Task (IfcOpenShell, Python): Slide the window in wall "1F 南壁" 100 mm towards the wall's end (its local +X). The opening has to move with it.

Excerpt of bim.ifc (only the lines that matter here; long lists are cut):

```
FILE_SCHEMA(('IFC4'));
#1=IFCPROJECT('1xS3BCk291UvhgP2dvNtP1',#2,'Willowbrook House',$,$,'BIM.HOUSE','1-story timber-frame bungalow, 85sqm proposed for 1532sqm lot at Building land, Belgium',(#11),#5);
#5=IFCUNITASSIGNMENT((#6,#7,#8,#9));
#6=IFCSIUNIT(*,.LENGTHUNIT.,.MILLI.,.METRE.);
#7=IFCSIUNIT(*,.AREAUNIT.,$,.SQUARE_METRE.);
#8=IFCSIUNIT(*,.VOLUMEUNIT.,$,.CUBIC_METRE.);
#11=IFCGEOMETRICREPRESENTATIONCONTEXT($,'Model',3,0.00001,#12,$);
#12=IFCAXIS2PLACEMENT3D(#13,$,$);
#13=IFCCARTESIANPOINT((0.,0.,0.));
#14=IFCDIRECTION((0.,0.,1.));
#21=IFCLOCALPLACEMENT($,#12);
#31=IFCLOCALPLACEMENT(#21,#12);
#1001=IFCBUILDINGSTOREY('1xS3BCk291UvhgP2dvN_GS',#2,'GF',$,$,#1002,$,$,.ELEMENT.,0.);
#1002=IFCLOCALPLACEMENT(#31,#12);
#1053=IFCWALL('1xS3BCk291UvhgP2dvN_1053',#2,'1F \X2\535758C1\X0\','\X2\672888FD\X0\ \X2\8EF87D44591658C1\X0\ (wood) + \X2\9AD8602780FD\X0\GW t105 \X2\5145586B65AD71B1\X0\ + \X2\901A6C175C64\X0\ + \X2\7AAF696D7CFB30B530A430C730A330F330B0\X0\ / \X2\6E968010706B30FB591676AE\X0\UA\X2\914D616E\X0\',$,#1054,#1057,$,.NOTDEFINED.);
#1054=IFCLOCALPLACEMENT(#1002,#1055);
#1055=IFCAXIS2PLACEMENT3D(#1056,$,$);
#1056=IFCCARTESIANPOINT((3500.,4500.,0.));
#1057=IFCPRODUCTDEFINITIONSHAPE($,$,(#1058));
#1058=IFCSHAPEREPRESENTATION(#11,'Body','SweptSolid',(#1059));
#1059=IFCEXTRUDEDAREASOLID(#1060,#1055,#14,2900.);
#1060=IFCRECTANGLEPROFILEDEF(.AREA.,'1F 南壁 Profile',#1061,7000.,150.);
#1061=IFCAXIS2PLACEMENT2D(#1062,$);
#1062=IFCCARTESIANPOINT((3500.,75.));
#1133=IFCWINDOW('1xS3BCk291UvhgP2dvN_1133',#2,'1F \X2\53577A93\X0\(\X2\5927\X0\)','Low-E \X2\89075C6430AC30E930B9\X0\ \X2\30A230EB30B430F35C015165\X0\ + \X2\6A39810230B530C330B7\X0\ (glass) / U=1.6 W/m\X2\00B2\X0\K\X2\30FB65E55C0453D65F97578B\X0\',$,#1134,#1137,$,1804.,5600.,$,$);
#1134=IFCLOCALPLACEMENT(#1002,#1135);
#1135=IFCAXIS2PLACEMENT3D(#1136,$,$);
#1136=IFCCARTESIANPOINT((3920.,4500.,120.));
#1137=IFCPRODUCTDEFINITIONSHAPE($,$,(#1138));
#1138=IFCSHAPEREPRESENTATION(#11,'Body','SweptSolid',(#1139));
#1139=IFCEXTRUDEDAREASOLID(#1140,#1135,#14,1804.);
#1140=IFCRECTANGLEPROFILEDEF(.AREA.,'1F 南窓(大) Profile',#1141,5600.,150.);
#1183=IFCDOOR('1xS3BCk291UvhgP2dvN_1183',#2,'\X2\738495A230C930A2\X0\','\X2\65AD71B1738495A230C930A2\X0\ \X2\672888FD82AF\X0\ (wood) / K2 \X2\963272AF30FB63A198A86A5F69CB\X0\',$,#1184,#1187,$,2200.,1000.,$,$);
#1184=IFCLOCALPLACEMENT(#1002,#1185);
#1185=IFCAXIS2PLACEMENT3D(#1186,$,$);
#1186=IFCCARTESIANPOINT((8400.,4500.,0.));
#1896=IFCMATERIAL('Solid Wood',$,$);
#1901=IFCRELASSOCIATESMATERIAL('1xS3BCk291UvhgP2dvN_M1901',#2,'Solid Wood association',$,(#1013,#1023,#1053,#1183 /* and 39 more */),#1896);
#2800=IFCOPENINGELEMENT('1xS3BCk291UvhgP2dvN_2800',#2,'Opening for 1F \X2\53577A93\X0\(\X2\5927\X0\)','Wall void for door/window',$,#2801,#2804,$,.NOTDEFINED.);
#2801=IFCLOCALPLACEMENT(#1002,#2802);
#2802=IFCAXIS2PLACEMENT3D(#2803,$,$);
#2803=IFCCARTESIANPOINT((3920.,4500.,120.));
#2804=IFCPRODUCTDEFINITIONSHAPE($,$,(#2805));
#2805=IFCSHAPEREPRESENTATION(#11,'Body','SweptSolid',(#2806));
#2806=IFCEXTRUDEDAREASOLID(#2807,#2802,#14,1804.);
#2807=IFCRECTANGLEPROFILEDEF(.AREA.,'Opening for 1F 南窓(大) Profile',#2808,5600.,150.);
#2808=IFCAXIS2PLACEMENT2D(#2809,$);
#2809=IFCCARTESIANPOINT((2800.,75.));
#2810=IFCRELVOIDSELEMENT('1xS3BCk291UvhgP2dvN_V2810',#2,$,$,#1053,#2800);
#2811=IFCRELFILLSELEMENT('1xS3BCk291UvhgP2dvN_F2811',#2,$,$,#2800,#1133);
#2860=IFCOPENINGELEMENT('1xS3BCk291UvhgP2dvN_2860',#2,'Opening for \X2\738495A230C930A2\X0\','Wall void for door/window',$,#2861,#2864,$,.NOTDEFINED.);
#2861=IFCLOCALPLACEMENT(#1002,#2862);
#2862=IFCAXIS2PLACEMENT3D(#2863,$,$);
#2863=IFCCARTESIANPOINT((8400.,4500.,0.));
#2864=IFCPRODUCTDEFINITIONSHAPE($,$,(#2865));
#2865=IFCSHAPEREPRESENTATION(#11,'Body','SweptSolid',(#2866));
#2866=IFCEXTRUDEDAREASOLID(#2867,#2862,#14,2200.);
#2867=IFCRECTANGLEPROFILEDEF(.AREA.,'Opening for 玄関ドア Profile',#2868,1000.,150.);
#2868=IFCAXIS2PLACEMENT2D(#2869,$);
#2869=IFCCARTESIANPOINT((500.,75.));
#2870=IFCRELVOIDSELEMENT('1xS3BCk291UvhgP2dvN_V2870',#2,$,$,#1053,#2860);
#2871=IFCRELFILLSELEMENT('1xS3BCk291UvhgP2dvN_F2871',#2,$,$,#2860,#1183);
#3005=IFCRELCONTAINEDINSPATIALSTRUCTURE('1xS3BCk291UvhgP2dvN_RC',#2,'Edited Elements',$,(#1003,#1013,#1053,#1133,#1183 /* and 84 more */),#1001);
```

```python
import ifcopenshell
import ifcopenshell.api.geometry
import ifcopenshell.util.placement
import ifcopenshell.util.unit

model = ifcopenshell.open("bim.ifc")
unit_scale = ifcopenshell.util.unit.calculate_unit_scale(model)

window = model.by_id(1133)
opening = window.FillsVoids[0].RelatingOpeningElement
wall = opening.VoidsElements[0].RelatingBuildingElement

wall_matrix = ifcopenshell.util.placement.get_local_placement(wall.ObjectPlacement)
shift = wall_matrix[:3, 0] * 0.1 / unit_scale
before = ifcopenshell.util.placement.get_local_placement(window.ObjectPlacement)[:3, 3].copy()

# The window is not placed relative to its opening, so move both.
for product in (opening, window):
    matrix = ifcopenshell.util.placement.get_local_placement(product.ObjectPlacement)
    matrix[:3, 3] += shift
    ifcopenshell.api.geometry.edit_object_placement(model, product=product, matrix=matrix, is_si=False)

after = ifcopenshell.util.placement.get_local_placement(window.ObjectPlacement)[:3, 3]
print("window moved by", (after - before).round(3) + 0.0)

model.write("bim_rev.ifc")
```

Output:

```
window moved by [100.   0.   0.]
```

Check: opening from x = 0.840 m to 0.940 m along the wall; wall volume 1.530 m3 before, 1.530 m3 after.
